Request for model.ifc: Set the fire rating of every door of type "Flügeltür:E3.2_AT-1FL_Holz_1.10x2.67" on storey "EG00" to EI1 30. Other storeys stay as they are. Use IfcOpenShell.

First a look at what the model holds.

```python
import ifcopenshell
import ifcopenshell.util.element

model = ifcopenshell.open("model.ifc")
print(model.schema)
storey = next(s for s in model.by_type("IfcBuildingStorey") if s.Name == "EG00")
doors = [e for e in ifcopenshell.util.element.get_decomposition(storey) if e.is_a("IfcDoor")]
seen = {}
for e in doors:
    element_type = ifcopenshell.util.element.get_type(e)
    key = (element_type.Name if element_type != e and element_type else None, ifcopenshell.util.element.get_pset(e, "Pset_DoorCommon", "FireRating"))
    seen[key] = seen.get(key, 0) + 1
for (name, value), count in sorted(seen.items(), key=str):
    print(count, "x", name, "|", value)
```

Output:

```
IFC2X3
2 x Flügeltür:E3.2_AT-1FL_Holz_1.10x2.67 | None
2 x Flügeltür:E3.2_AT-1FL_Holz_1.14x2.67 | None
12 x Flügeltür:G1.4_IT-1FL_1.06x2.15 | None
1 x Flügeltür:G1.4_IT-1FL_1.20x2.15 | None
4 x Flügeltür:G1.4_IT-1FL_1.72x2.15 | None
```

```python
import ifcopenshell
import ifcopenshell.api.pset
import ifcopenshell.util.element

model = ifcopenshell.open("model.ifc")

storey = next(s for s in model.by_type("IfcBuildingStorey") if s.Name == "EG00")
doors = [e for e in ifcopenshell.util.element.get_decomposition(storey) if e.is_a("IfcDoor")]

count = 0
for e in doors:
    element_type = ifcopenshell.util.element.get_type(e)
    if element_type in (None, e) or element_type.Name != "Flügeltür:E3.2_AT-1FL_Holz_1.10x2.67":
        continue
    # add_pset returns the element's existing set when there is one.
    pset = ifcopenshell.api.pset.add_pset(model, product=e, name="Pset_DoorCommon")
    ifcopenshell.api.pset.edit_pset(model, pset=pset, properties={"FireRating": "EI1 30"})
    count += 1

print(count, "doors updated")

model.write("model_v2.ifc")
```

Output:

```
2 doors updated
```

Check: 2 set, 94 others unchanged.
